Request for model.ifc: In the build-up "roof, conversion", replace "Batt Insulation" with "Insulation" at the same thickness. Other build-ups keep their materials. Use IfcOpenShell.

First a look at what the model holds.

```python
import ifcopenshell
import ifcopenshell.util.element

model = ifcopenshell.open("model.ifc")
print(model.schema)
for layer_set in model.by_type("IfcMaterialLayerSet"):
    if layer_set.LayerSetName == "roof, conversion":
        for layer in layer_set.MaterialLayers:
            print(layer.id(), layer.Material and layer.Material.Name, layer.LayerThickness, sep=" | ")
        print(len(ifcopenshell.util.element.get_elements_by_material(model, layer_set)), "elements and types use it")
print(sorted(m.Name for m in model.by_type("IfcMaterial") if m.Name)[:60])
```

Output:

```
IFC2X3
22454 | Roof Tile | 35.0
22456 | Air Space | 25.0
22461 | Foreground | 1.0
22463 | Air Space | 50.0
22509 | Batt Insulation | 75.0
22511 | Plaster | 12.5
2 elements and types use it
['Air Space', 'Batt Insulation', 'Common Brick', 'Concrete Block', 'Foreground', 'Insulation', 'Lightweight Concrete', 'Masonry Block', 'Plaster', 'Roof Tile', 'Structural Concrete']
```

```python
import ifcopenshell
import ifcopenshell.api.material

model = ifcopenshell.open("model.ifc")

layer_set = next(s for s in model.by_type("IfcMaterialLayerSet") if s.LayerSetName == "roof, conversion")
layer = next(l for l in layer_set.MaterialLayers if l.Material and l.Material.Name == "Batt Insulation")
material = next(m for m in model.by_type("IfcMaterial") if m.Name == "Insulation")

# Point this one layer at the other material; renaming the old one would change it everywhere.
ifcopenshell.api.material.edit_layer(model, layer=layer, attributes={}, material=material)

print([l.Material.Name if l.Material else None for l in layer_set.MaterialLayers])

model.write("model_updated.ifc")
```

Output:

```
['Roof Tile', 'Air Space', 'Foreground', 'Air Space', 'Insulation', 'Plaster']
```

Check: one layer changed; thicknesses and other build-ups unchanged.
